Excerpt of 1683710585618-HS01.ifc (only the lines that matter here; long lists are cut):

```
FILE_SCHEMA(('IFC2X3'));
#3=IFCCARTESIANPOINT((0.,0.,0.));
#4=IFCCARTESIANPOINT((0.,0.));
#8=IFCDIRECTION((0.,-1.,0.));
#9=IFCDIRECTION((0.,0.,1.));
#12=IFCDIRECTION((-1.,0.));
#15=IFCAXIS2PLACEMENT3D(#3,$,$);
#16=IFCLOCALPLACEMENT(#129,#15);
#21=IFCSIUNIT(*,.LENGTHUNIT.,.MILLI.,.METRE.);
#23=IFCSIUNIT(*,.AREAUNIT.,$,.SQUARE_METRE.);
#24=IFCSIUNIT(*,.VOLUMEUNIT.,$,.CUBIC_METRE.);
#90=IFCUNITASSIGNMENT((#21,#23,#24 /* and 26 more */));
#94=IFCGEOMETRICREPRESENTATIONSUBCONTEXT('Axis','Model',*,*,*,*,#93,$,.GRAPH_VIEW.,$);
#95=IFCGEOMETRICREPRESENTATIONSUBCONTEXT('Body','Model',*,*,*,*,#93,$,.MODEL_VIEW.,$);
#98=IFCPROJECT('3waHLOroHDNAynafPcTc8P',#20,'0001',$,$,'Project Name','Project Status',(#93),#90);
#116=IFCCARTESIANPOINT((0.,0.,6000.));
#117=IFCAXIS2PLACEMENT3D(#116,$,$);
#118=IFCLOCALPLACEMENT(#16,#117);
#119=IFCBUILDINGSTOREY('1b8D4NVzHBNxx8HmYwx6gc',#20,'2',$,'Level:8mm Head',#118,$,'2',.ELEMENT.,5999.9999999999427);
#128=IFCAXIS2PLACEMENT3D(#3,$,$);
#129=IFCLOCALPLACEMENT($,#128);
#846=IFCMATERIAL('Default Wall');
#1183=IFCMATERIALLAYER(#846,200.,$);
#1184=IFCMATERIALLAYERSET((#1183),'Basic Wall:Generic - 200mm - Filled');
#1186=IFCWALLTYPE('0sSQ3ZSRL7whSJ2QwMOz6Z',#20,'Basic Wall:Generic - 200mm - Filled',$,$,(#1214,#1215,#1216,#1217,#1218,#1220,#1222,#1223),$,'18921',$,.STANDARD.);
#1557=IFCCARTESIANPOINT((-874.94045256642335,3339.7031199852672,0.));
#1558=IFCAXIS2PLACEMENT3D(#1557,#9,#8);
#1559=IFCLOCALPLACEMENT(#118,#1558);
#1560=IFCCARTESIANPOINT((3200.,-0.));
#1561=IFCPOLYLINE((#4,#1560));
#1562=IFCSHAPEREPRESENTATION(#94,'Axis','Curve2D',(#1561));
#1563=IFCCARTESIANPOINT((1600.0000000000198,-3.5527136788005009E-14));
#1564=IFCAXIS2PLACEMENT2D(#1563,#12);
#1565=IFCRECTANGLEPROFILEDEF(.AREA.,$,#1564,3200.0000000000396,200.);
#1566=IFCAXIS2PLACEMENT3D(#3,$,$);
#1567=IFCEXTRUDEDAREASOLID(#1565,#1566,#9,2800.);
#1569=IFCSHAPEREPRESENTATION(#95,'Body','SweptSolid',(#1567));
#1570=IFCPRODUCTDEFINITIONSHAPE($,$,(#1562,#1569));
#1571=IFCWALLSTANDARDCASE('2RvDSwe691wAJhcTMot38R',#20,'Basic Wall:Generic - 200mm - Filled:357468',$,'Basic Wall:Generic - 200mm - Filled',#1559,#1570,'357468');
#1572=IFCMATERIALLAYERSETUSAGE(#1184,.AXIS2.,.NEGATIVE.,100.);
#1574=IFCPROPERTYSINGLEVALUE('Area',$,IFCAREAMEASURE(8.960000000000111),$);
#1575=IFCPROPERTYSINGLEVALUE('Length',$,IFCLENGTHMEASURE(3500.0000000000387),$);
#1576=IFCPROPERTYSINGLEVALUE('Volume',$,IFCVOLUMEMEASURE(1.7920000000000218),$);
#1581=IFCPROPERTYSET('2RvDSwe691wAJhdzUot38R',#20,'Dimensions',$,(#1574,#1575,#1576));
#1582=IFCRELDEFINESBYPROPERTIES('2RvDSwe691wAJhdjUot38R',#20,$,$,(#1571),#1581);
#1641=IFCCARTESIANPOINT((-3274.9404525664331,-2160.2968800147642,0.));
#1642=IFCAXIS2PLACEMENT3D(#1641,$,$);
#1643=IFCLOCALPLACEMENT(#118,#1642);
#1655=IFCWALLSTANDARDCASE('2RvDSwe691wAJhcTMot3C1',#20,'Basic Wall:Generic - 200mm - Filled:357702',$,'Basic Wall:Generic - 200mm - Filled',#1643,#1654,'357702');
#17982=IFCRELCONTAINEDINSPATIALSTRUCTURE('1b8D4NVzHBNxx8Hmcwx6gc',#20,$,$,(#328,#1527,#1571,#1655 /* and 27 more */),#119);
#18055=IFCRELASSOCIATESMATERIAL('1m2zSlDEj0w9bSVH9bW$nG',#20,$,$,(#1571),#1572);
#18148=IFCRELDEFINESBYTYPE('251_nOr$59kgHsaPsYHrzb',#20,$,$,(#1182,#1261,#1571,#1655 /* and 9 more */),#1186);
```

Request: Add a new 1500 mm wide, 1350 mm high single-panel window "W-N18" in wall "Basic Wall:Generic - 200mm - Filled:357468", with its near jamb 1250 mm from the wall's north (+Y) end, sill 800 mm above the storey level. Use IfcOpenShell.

```python
import numpy as np
import ifcopenshell
import ifcopenshell.api.feature
import ifcopenshell.api.geometry
import ifcopenshell.api.pset
import ifcopenshell.api.root
import ifcopenshell.api.spatial
import ifcopenshell.api.type
import ifcopenshell.geom
import ifcopenshell.util.element
import ifcopenshell.util.placement
import ifcopenshell.util.representation
import ifcopenshell.util.shape
import ifcopenshell.util.unit

model = ifcopenshell.open("1683710585618-HS01.ifc")
unit_scale = ifcopenshell.util.unit.calculate_unit_scale(model)
area_scale = ifcopenshell.util.unit.calculate_unit_scale(model, "AREAUNIT")
volume_scale = ifcopenshell.util.unit.calculate_unit_scale(model, "VOLUMEUNIT")
settings = ifcopenshell.geom.settings()


def volume(element):
    """Net volume in cubic metres, openings subtracted."""
    shape = ifcopenshell.geom.create_shape(settings, element)
    return ifcopenshell.util.shape.get_volume(shape.geometry)


wall = model.by_guid("2RvDSwe691wAJhcTMot38R")
storey = ifcopenshell.util.element.get_container(wall, ifc_class="IfcBuildingStorey")
context = ifcopenshell.util.representation.get_context(model, "Model", "Body", "MODEL_VIEW")
before = volume(wall)

width, height, from_end, sill = 1.5, 1.35, 1.25, 0.8  # metres

# The wall runs along its own X axis, and the end named is its -X end.
wall_shape = ifcopenshell.geom.create_shape(settings, wall)
x, y, z = ifcopenshell.util.shape.get_vertices(wall_shape.geometry).T
start = x.min() + from_end
face, thickness = float(y.min()), float(y.max() - y.min())
wall_matrix = ifcopenshell.util.placement.get_local_placement(wall.ObjectPlacement)
level = ifcopenshell.util.placement.get_local_placement(storey.ObjectPlacement)[2, 3]


def in_wall(x, y):
    """Placement at x, y metres in the wall's axes, at sill height."""
    matrix = wall_matrix.copy()
    matrix[:, 3] = wall_matrix @ np.array([x / unit_scale, y / unit_scale, 0.0, 1.0])
    matrix[2, 3] = level + sill / unit_scale
    return matrix


# Opening: a box that overshoots both wall faces by 50 mm.
opening = ifcopenshell.api.root.create_entity(model, ifc_class="IfcOpeningElement")
box = ifcopenshell.api.geometry.add_wall_representation(
    model, context=context, length=width, height=height, thickness=thickness + 0.1
)
ifcopenshell.api.geometry.assign_representation(model, product=opening, representation=box)
ifcopenshell.api.geometry.edit_object_placement(model, product=opening, matrix=in_wall(start, face - 0.05), is_si=False)
ifcopenshell.api.feature.add_feature(model, feature=opening, element=wall)

window = ifcopenshell.api.root.create_entity(model, ifc_class="IfcWindow", name="W-N18")
window.OverallWidth, window.OverallHeight = width / unit_scale, height / unit_scale
body = ifcopenshell.api.geometry.add_window_representation(
    model,
    context=context,
    overall_width=window.OverallWidth,
    overall_height=window.OverallHeight,
    partition_type="SINGLE_PANEL",
)
ifcopenshell.api.geometry.assign_representation(model, product=window, representation=body)
ifcopenshell.api.spatial.assign_container(model, products=[window], relating_structure=storey)
fills = ifcopenshell.api.feature.add_filling(model, opening=opening, element=window)
fills.OwnerHistory = window.OwnerHistory  # required in IFC2X3

# IFC2X3 keeps the operation on the window style.
style = ifcopenshell.api.root.create_entity(model, ifc_class="IfcWindowStyle", name="W-N18")
style.OperationType, style.ConstructionType = "SINGLE_PANEL", "NOTDEFINED"
style.ParameterTakesPrecedence = style.Sizeable = False
ifcopenshell.api.type.assign_type(model, related_objects=[window], relating_type=style)

# Centre the window in the wall's thickness.
ifcopenshell.api.geometry.edit_object_placement(model, product=window, matrix=in_wall(start, face), is_si=False)
window_shape = ifcopenshell.geom.create_shape(settings, window)
depth = ifcopenshell.util.shape.get_vertices(window_shape.geometry)[:, 1]
offset = face + thickness / 2 - (depth.min() + depth.max()) / 2
ifcopenshell.api.geometry.edit_object_placement(model, product=window, matrix=in_wall(start, offset), is_si=False)

after = volume(wall)

# Update the wall's stored quantities.
pset = model.by_id(ifcopenshell.util.element.get_pset(wall, "Dimensions", should_inherit=False)["id"])
ifcopenshell.api.pset.edit_pset(model, pset=pset, properties={
    "Area": model.create_entity("IfcAreaMeasure", after / thickness / area_scale),
    "Volume": model.create_entity("IfcVolumeMeasure", after / volume_scale),
})

print(f"wall volume {before:.3f} -> {after:.3f} m3")

model.write("1683710585618-HS01_updated.ifc")
```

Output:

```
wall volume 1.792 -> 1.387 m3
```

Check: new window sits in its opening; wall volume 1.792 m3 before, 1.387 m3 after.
